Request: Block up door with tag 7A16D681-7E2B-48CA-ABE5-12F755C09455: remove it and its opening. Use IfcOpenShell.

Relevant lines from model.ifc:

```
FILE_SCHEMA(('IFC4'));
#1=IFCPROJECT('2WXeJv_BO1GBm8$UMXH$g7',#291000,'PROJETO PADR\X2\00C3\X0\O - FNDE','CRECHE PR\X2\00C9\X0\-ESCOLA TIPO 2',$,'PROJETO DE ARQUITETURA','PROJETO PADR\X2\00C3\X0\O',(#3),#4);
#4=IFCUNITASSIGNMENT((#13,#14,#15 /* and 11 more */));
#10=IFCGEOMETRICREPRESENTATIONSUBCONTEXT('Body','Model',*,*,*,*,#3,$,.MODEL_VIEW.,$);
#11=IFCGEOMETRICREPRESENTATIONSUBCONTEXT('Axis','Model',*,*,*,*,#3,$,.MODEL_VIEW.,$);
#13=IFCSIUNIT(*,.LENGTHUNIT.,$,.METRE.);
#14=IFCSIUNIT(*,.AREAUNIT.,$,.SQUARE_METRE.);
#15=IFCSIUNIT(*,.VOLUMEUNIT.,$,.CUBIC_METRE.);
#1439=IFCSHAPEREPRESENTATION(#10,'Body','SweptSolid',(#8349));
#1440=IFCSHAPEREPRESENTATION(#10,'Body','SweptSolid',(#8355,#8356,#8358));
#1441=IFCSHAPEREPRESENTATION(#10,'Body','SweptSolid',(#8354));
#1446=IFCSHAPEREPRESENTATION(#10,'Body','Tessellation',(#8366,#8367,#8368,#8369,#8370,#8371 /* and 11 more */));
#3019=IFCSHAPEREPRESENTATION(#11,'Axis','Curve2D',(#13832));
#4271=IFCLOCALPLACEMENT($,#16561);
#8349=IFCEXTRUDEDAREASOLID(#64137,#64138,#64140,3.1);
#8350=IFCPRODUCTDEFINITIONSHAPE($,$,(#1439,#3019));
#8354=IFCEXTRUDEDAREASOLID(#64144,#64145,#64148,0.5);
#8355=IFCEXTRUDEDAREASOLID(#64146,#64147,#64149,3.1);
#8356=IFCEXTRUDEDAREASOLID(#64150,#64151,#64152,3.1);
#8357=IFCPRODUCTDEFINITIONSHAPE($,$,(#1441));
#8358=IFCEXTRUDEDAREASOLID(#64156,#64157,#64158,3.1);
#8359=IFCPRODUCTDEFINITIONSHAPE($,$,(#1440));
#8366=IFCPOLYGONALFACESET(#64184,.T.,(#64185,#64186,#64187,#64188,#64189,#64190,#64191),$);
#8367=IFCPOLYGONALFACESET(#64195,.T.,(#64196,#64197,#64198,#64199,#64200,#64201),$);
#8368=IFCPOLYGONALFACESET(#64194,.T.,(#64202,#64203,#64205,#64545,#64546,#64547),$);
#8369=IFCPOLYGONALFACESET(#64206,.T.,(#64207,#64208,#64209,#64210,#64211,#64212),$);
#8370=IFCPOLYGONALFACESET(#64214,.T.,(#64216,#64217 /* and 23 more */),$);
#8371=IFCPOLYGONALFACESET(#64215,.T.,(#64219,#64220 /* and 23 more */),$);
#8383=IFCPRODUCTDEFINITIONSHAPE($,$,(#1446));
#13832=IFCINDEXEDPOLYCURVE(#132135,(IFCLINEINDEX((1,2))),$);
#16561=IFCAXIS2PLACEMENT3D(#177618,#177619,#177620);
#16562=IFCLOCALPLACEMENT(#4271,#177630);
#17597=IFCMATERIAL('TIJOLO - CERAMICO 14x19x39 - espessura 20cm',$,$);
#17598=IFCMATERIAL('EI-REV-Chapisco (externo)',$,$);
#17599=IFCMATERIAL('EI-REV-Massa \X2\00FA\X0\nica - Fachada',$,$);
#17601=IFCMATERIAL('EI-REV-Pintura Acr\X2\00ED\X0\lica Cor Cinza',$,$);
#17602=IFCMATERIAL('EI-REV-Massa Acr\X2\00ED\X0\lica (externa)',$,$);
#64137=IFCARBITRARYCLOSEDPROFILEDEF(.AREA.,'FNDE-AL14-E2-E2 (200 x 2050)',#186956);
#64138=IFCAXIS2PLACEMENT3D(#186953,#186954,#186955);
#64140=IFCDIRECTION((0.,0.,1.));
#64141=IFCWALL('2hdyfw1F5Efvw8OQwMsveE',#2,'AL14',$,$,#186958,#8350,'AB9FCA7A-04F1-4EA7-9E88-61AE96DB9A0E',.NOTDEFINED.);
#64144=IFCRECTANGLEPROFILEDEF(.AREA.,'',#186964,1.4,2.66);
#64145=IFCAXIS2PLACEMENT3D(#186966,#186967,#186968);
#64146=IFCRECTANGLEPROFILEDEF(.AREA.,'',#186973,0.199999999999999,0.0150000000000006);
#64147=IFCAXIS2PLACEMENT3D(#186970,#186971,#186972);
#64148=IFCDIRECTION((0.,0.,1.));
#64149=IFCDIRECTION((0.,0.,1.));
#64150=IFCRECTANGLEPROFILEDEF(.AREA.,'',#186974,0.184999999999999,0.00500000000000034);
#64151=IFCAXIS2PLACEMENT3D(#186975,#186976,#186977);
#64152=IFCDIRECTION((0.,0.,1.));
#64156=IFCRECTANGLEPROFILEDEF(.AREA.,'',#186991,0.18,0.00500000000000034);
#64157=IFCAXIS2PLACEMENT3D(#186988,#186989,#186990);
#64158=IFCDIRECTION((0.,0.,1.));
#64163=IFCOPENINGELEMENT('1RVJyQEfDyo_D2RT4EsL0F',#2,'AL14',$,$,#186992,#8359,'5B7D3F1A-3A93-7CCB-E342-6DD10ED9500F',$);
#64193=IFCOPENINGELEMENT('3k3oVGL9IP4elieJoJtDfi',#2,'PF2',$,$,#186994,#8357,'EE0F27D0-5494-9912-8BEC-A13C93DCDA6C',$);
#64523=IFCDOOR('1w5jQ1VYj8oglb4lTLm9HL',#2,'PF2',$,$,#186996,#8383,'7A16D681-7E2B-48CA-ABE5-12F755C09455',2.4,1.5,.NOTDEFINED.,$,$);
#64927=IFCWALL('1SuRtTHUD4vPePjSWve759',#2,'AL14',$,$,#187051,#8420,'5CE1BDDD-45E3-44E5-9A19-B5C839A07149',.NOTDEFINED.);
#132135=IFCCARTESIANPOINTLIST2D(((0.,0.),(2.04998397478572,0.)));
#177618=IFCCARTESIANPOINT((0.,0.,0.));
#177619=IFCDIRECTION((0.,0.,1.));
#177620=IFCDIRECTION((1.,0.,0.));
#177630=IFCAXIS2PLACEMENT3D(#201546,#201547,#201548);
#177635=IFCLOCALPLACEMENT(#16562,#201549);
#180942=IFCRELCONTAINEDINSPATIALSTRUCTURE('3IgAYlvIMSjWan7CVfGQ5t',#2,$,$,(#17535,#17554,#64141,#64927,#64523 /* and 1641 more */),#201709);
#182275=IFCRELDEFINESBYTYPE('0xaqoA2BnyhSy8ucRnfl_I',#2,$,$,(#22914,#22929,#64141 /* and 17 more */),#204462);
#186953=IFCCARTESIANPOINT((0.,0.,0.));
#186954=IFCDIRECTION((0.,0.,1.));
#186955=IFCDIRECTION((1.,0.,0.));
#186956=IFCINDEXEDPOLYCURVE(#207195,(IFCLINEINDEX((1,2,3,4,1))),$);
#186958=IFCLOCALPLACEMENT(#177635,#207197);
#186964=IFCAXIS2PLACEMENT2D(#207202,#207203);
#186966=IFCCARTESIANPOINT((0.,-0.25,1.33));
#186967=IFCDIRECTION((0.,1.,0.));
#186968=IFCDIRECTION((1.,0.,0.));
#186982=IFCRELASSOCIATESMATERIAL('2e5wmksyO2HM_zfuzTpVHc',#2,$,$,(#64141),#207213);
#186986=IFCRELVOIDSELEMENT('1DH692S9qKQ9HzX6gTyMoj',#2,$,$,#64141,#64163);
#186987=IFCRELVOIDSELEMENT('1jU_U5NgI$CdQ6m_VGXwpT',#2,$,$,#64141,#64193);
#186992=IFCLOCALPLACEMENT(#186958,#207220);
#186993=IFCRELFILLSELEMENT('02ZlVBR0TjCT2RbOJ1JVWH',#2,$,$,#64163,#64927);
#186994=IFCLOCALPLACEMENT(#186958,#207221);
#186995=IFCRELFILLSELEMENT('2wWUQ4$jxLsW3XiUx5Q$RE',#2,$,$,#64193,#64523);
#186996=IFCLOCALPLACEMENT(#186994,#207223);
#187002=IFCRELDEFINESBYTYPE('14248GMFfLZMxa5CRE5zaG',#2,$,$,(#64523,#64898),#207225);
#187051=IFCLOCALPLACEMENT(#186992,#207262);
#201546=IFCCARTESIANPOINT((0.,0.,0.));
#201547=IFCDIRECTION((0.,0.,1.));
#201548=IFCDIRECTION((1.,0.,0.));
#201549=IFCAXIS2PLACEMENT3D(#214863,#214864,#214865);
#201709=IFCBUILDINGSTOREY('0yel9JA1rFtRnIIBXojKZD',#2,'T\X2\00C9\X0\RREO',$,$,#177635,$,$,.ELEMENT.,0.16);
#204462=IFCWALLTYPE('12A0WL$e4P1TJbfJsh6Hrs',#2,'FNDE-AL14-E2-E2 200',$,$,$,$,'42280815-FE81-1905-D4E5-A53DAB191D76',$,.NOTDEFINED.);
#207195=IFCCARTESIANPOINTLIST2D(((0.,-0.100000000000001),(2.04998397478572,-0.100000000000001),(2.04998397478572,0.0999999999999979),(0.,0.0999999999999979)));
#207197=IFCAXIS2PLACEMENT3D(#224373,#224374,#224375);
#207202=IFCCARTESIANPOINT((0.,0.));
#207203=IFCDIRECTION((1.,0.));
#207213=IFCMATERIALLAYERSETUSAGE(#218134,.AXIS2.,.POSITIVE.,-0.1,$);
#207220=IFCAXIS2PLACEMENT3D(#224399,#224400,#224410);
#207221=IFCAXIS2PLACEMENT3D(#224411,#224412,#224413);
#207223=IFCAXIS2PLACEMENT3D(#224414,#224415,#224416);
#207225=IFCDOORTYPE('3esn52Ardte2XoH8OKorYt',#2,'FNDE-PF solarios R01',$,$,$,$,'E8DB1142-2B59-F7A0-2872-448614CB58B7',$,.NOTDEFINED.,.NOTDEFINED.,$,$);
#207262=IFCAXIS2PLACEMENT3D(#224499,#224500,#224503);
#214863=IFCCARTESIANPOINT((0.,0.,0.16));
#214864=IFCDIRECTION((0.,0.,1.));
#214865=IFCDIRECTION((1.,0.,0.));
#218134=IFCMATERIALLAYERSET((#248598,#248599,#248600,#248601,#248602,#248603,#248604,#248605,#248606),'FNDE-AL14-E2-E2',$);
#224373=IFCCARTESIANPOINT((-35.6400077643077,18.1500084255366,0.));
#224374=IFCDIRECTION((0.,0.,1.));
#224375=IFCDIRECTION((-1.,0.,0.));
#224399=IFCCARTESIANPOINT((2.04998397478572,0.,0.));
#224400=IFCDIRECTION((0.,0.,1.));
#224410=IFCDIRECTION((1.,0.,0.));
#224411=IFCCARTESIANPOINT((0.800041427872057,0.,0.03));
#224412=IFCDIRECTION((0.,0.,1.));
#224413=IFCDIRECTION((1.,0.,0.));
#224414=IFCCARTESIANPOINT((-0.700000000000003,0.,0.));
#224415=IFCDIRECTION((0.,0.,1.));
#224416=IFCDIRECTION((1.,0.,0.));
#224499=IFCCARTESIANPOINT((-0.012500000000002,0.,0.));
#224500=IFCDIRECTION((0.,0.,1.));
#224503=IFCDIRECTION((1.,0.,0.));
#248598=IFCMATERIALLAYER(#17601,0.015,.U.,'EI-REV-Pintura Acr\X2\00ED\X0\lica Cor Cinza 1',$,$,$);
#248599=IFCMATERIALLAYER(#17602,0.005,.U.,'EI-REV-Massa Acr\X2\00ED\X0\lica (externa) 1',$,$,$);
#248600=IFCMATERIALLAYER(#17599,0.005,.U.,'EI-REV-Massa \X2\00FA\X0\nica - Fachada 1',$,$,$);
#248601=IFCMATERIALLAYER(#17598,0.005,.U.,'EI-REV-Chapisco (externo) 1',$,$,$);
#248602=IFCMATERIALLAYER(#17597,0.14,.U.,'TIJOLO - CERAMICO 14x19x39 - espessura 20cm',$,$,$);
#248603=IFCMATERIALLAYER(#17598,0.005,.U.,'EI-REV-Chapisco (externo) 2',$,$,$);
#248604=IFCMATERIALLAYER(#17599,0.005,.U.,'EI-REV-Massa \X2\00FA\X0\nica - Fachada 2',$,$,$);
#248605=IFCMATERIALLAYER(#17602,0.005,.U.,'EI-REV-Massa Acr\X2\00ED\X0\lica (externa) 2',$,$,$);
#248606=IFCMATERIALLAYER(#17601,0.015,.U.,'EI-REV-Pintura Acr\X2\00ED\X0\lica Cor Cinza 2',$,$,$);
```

```python
import ifcopenshell
import ifcopenshell.api.feature
import ifcopenshell.api.root
import ifcopenshell.geom
import ifcopenshell.util.shape

model = ifcopenshell.open("model.ifc")
settings = ifcopenshell.geom.settings()


def volume(element):
    """Net volume in cubic metres, openings subtracted."""
    shape = ifcopenshell.geom.create_shape(settings, element)
    return ifcopenshell.util.shape.get_volume(shape.geometry)


door = model.by_guid("1w5jQ1VYj8oglb4lTLm9HL")
opening = door.FillsVoids[0].RelatingOpeningElement
wall = opening.VoidsElements[0].RelatingBuildingElement
before = volume(wall)

ifcopenshell.api.root.remove_product(model, product=door)
ifcopenshell.api.feature.remove_feature(model, feature=opening)

after = volume(wall)

print(f"wall volume {before:.3f} -> {after:.3f} m3")

model.write("model_updated.ifc")
```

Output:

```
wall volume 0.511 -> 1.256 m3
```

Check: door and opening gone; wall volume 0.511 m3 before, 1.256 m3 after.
